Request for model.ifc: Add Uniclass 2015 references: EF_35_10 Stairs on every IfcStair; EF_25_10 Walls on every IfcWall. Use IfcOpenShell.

First a look at what the model holds.

```python
import ifcopenshell

model = ifcopenshell.open("model.ifc")
print(model.schema)
print("classifications:", [c.Name for c in model.by_type("IfcClassification")])
for ifc_class in ("IfcDoor", "IfcRoof", "IfcStair", "IfcWall", "IfcWindow"):
    print(ifc_class, len(model.by_type(ifc_class)))
```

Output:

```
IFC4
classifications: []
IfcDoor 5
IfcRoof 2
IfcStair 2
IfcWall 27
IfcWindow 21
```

```python
import ifcopenshell
import ifcopenshell.api.classification

model = ifcopenshell.open("model.ifc")

system = ifcopenshell.api.classification.add_classification(model, classification="Uniclass 2015")

codes = {
    "IfcStair": ("EF_35_10", "Stairs"),
    "IfcWall": ("EF_25_10", "Walls"),
}
for ifc_class, (code, name) in codes.items():
    products = model.by_type(ifc_class)
    ifcopenshell.api.classification.add_reference(
        model, products=products, classification=system, identification=code, name=name
    )
    print(code, len(products))

model.write("model_edited.ifc")
```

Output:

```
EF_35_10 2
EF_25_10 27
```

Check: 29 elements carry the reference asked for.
